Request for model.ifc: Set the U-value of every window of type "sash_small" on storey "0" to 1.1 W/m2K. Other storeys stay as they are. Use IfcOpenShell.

First a look at what the model holds.

```python
import ifcopenshell
import ifcopenshell.util.element

model = ifcopenshell.open("model.ifc")
print(model.schema)
storey = next(s for s in model.by_type("IfcBuildingStorey") if s.Name == "0")
windows = [e for e in ifcopenshell.util.element.get_decomposition(storey) if e.is_a("IfcWindow")]
seen = {}
for e in windows:
    element_type = ifcopenshell.util.element.get_type(e)
    key = (element_type.Name if element_type != e and element_type else None, ifcopenshell.util.element.get_pset(e, "Pset_WindowCommon", "ThermalTransmittance"))
    seen[key] = seen.get(key, 0) + 1
for (name, value), count in sorted(seen.items(), key=str):
    print(count, "x", name, "|", value)
```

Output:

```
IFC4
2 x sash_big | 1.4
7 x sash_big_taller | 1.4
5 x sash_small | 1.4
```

```python
import ifcopenshell
import ifcopenshell.api.pset
import ifcopenshell.util.element

model = ifcopenshell.open("model.ifc")

storey = next(s for s in model.by_type("IfcBuildingStorey") if s.Name == "0")
windows = [e for e in ifcopenshell.util.element.get_decomposition(storey) if e.is_a("IfcWindow")]

count = 0
for e in windows:
    element_type = ifcopenshell.util.element.get_type(e)
    if element_type in (None, e) or element_type.Name != "sash_small":
        continue
    # add_pset returns the element's existing set when there is one.
    pset = ifcopenshell.api.pset.add_pset(model, product=e, name="Pset_WindowCommon")
    ifcopenshell.api.pset.edit_pset(model, pset=pset, properties={"ThermalTransmittance": 1.1})
    count += 1

print(count, "windows updated")

model.write("model_rev.ifc")
```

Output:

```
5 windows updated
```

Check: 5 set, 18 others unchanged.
